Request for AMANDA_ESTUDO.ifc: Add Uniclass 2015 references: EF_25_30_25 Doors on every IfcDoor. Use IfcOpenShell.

First a look at what the model holds.

```python
import ifcopenshell

model = ifcopenshell.open("AMANDA_ESTUDO.ifc")
print(model.schema)
print("classifications:", [c.Name for c in model.by_type("IfcClassification")])
for ifc_class in ("IfcDoor", "IfcRoof", "IfcStair", "IfcWall", "IfcWindow"):
    print(ifc_class, len(model.by_type(ifc_class)))
```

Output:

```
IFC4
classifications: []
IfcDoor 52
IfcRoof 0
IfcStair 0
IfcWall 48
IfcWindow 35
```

```python
import ifcopenshell
import ifcopenshell.api.classification

model = ifcopenshell.open("AMANDA_ESTUDO.ifc")

system = ifcopenshell.api.classification.add_classification(model, classification="Uniclass 2015")

codes = {
    "IfcDoor": ("EF_25_30_25", "Doors"),
}
for ifc_class, (code, name) in codes.items():
    products = model.by_type(ifc_class)
    ifcopenshell.api.classification.add_reference(
        model, products=products, classification=system, identification=code, name=name
    )
    print(code, len(products))

model.write("AMANDA_ESTUDO_rev.ifc")
```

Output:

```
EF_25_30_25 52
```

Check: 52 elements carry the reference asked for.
